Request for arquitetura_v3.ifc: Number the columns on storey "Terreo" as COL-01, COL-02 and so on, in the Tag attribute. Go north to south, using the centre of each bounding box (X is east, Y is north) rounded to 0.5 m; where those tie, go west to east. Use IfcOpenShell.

First a look at what the model holds.

```python
import ifcopenshell
import ifcopenshell.util.element
import ifcopenshell.util.placement

model = ifcopenshell.open("arquitetura_v3.ifc")
print(model.schema)
storey = next(s for s in model.by_type("IfcBuildingStorey") if s.Name == "Terreo")
columns = [e for e in ifcopenshell.util.element.get_decomposition(storey) if e.is_a("IfcColumn")]
for e in sorted(columns, key=lambda e: e.id()):
    origin = ifcopenshell.util.placement.get_local_placement(e.ObjectPlacement)[:3, 3]
    print(e.id(), e.Tag, e.Name, origin.round(2) + 0.0, sep=" | ")
```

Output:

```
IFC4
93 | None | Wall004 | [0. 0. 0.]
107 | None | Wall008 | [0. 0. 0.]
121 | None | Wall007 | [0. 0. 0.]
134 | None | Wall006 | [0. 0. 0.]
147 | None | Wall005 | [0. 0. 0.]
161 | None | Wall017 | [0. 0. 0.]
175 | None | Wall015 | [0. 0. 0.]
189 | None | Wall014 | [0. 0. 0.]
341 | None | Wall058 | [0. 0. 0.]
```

```python
import ifcopenshell
import ifcopenshell.geom
import ifcopenshell.util.element
import ifcopenshell.util.shape

model = ifcopenshell.open("arquitetura_v3.ifc")
settings = ifcopenshell.geom.settings()
settings.set("use-world-coords", True)


def centre(element):
    shape = ifcopenshell.geom.create_shape(settings, element)
    return ifcopenshell.util.shape.get_bbox_centroid(shape.geometry)


storey = next(s for s in model.by_type("IfcBuildingStorey") if s.Name == "Terreo")
columns = [e for e in ifcopenshell.util.element.get_decomposition(storey) if e.is_a("IfcColumn")]

# Insertion points can sit at a corner or the storey origin, so sort by the geometry (in metres).
centres = {e: centre(e) for e in columns}
columns.sort(key=lambda e: (-round(centres[e][1] / 0.5), centres[e][0]))

for i, e in enumerate(columns, start=1):
    number = f"COL-{i:02d}"
    e.Tag = number
    print(e.id(), number)

model.write("arquitetura_v3_rev.ifc")
```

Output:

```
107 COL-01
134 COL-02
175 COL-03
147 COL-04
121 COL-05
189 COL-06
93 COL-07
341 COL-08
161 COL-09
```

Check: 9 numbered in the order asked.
